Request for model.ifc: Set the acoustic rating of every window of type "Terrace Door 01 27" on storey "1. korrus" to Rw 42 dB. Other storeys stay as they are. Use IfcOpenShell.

First a look at what the model holds.

```python
import ifcopenshell
import ifcopenshell.util.element

model = ifcopenshell.open("model.ifc")
print(model.schema)
storey = next(s for s in model.by_type("IfcBuildingStorey") if s.Name == "1. korrus")
windows = [e for e in ifcopenshell.util.element.get_decomposition(storey) if e.is_a("IfcWindow")]
seen = {}
for e in windows:
    element_type = ifcopenshell.util.element.get_type(e)
    key = (element_type.Name if element_type != e and element_type else None, ifcopenshell.util.element.get_pset(e, "Pset_WindowCommon", "AcousticRating"))
    seen[key] = seen.get(key, 0) + 1
for (name, value), count in sorted(seen.items(), key=str):
    print(count, "x", name, "|", value)
```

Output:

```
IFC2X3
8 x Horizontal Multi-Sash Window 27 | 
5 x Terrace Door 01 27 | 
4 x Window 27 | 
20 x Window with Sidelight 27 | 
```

```python
import ifcopenshell
import ifcopenshell.api.pset
import ifcopenshell.util.element

model = ifcopenshell.open("model.ifc")

storey = next(s for s in model.by_type("IfcBuildingStorey") if s.Name == "1. korrus")
windows = [e for e in ifcopenshell.util.element.get_decomposition(storey) if e.is_a("IfcWindow")]

count = 0
for e in windows:
    element_type = ifcopenshell.util.element.get_type(e)
    if element_type in (None, e) or element_type.Name != "Terrace Door 01 27":
        continue
    # add_pset returns the element's existing set when there is one.
    pset = ifcopenshell.api.pset.add_pset(model, product=e, name="Pset_WindowCommon")
    ifcopenshell.api.pset.edit_pset(model, pset=pset, properties={"AcousticRating": "Rw 42 dB"})
    count += 1

print(count, "windows updated")

model.write("model_rev.ifc")
```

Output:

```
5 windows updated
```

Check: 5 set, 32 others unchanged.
